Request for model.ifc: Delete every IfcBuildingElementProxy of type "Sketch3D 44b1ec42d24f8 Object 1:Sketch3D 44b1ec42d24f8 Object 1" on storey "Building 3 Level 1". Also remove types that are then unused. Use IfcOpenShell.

First a look at what the model holds.

```python
import ifcopenshell
import ifcopenshell.util.element

model = ifcopenshell.open("model.ifc")
print(model.schema)
storey = next(s for s in model.by_type("IfcBuildingStorey") if s.Name == "Building 3 Level 1")
proxies = [e for e in ifcopenshell.util.element.get_decomposition(storey) if e.is_a("IfcBuildingElementProxy")]
seen = {}
for e in proxies:
    element_type = ifcopenshell.util.element.get_type(e)
    name = element_type.Name if element_type not in (None, e) else None
    seen[name] = seen.get(name, 0) + 1
for name, count in sorted(seen.items(), key=str):
    print(count, "x", name)
```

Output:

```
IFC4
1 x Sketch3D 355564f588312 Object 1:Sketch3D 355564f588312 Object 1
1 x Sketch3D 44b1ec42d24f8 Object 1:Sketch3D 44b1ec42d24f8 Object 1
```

```python
import ifcopenshell
import ifcopenshell.api.root
import ifcopenshell.util.element

model = ifcopenshell.open("model.ifc")

storey = next(s for s in model.by_type("IfcBuildingStorey") if s.Name == "Building 3 Level 1")
proxies = [e for e in ifcopenshell.util.element.get_decomposition(storey) if e.is_a("IfcBuildingElementProxy")]
targets = [e for e in proxies if (t := ifcopenshell.util.element.get_type(e)) not in (None, e) and t.Name == "Sketch3D 44b1ec42d24f8 Object 1:Sketch3D 44b1ec42d24f8 Object 1"]
types = {ifcopenshell.util.element.get_type(e) for e in targets} - {None, *targets}

for e in targets:
    ifcopenshell.api.root.remove_product(model, product=e)
print(len(targets), "removed")

unused = [t for t in types if not ifcopenshell.util.element.get_types(t)]
for t in unused:
    ifcopenshell.api.root.remove_product(model, product=t)
print(len(unused), "unused types removed")

model.write("model_v2.ifc")
```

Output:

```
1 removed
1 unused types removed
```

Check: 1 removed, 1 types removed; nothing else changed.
